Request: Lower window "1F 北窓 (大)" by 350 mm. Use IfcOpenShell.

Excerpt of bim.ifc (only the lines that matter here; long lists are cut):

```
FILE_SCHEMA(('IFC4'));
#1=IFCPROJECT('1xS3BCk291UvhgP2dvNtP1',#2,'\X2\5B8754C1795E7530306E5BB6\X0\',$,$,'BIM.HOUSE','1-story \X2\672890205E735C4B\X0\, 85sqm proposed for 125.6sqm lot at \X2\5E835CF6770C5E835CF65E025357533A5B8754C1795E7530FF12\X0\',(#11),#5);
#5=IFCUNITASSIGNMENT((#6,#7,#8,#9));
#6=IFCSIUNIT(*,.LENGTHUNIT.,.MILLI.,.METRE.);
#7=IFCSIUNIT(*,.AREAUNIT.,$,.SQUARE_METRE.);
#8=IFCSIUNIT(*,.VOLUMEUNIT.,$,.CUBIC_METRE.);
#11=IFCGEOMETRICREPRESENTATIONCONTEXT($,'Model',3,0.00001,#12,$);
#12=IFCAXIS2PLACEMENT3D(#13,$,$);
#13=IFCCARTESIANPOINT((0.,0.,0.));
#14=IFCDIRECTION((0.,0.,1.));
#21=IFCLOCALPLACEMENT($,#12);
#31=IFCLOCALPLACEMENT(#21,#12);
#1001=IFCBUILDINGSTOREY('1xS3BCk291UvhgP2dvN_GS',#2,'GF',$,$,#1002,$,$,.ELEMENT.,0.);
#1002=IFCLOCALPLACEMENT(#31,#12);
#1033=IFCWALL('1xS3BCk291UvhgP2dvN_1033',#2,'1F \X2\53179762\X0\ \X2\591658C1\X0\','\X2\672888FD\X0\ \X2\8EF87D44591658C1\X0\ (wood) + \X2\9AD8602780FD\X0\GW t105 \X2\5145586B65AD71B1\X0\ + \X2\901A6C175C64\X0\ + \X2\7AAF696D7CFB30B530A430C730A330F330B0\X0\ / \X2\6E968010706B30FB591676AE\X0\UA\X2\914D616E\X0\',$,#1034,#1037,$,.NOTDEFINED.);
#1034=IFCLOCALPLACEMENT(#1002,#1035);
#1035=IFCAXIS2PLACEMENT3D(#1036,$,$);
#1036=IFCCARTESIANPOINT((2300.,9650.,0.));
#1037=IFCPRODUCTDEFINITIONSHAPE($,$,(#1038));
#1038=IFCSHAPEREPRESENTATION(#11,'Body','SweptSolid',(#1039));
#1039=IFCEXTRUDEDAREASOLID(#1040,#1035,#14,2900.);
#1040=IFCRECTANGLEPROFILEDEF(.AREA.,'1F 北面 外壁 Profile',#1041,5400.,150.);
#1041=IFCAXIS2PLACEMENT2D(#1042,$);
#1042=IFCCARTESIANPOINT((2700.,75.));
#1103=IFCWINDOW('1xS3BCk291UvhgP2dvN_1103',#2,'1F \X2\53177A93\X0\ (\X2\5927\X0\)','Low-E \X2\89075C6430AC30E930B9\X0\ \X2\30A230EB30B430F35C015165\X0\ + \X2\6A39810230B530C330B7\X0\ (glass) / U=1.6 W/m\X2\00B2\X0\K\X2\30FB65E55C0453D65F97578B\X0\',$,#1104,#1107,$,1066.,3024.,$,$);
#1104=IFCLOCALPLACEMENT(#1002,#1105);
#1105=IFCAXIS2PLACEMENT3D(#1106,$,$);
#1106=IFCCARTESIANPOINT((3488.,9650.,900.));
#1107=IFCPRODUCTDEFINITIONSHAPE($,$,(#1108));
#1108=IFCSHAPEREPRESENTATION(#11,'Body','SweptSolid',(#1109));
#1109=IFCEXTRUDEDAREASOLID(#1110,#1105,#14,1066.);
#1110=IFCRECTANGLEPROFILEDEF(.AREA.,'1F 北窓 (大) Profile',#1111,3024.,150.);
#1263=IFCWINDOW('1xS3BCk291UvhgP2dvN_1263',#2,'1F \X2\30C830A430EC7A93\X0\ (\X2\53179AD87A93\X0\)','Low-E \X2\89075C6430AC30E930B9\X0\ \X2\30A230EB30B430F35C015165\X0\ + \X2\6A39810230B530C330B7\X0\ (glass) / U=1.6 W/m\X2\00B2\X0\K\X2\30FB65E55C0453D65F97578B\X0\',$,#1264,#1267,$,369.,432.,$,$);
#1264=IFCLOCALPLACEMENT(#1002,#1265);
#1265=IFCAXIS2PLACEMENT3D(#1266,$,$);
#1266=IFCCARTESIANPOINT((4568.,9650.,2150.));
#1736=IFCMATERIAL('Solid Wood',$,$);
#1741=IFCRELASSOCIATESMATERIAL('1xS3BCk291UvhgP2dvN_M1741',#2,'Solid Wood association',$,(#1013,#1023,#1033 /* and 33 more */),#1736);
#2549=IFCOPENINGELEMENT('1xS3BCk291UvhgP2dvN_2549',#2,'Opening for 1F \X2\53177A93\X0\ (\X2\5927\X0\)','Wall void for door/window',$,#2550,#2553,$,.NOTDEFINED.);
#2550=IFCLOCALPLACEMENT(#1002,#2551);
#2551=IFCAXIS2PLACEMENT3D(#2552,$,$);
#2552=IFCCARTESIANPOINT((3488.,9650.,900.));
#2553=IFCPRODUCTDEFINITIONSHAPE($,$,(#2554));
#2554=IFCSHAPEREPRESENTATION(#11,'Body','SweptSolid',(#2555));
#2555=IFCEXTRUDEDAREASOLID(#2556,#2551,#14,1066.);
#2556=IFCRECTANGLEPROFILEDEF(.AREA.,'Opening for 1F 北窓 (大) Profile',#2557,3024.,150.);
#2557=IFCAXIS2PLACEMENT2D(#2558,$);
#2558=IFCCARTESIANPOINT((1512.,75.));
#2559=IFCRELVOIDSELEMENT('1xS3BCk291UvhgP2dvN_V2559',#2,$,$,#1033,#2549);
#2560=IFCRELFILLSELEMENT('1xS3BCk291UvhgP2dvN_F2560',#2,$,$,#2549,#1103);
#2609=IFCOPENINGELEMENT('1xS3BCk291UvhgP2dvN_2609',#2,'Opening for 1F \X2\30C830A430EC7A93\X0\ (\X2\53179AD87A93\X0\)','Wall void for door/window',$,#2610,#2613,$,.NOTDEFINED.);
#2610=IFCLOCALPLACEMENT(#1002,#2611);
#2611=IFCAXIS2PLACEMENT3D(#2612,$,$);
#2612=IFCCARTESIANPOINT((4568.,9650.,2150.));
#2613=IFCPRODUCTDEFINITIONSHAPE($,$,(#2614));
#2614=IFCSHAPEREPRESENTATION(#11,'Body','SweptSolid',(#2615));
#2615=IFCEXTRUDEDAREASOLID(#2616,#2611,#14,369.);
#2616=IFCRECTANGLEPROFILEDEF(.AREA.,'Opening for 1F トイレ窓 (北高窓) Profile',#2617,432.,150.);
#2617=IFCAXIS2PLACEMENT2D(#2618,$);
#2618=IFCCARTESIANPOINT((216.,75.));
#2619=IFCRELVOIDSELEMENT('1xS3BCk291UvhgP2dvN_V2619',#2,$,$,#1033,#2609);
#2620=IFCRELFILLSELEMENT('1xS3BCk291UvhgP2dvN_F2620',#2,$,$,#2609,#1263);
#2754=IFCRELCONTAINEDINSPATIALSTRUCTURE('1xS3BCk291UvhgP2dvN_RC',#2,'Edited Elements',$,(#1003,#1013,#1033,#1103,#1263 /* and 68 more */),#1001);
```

```python
import numpy as np
import ifcopenshell
import ifcopenshell.api.geometry
import ifcopenshell.util.placement
import ifcopenshell.util.unit

model = ifcopenshell.open("bim.ifc")
unit_scale = ifcopenshell.util.unit.calculate_unit_scale(model)

window = model.by_id(1103)
opening = window.FillsVoids[0].RelatingOpeningElement
dz = -0.35 / unit_scale

shift = np.array([0.0, 0.0, dz])
# The window is not placed relative to its opening, so move both.
for product in (opening, window):
    matrix = ifcopenshell.util.placement.get_local_placement(product.ObjectPlacement)
    matrix[:3, 3] += shift
    ifcopenshell.api.geometry.edit_object_placement(model, product=product, matrix=matrix, is_si=False)

print(f"moved by {dz * unit_scale:+.3f} m")

model.write("bim_rev.ifc")
```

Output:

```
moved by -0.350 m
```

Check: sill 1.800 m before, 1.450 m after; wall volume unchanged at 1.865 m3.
